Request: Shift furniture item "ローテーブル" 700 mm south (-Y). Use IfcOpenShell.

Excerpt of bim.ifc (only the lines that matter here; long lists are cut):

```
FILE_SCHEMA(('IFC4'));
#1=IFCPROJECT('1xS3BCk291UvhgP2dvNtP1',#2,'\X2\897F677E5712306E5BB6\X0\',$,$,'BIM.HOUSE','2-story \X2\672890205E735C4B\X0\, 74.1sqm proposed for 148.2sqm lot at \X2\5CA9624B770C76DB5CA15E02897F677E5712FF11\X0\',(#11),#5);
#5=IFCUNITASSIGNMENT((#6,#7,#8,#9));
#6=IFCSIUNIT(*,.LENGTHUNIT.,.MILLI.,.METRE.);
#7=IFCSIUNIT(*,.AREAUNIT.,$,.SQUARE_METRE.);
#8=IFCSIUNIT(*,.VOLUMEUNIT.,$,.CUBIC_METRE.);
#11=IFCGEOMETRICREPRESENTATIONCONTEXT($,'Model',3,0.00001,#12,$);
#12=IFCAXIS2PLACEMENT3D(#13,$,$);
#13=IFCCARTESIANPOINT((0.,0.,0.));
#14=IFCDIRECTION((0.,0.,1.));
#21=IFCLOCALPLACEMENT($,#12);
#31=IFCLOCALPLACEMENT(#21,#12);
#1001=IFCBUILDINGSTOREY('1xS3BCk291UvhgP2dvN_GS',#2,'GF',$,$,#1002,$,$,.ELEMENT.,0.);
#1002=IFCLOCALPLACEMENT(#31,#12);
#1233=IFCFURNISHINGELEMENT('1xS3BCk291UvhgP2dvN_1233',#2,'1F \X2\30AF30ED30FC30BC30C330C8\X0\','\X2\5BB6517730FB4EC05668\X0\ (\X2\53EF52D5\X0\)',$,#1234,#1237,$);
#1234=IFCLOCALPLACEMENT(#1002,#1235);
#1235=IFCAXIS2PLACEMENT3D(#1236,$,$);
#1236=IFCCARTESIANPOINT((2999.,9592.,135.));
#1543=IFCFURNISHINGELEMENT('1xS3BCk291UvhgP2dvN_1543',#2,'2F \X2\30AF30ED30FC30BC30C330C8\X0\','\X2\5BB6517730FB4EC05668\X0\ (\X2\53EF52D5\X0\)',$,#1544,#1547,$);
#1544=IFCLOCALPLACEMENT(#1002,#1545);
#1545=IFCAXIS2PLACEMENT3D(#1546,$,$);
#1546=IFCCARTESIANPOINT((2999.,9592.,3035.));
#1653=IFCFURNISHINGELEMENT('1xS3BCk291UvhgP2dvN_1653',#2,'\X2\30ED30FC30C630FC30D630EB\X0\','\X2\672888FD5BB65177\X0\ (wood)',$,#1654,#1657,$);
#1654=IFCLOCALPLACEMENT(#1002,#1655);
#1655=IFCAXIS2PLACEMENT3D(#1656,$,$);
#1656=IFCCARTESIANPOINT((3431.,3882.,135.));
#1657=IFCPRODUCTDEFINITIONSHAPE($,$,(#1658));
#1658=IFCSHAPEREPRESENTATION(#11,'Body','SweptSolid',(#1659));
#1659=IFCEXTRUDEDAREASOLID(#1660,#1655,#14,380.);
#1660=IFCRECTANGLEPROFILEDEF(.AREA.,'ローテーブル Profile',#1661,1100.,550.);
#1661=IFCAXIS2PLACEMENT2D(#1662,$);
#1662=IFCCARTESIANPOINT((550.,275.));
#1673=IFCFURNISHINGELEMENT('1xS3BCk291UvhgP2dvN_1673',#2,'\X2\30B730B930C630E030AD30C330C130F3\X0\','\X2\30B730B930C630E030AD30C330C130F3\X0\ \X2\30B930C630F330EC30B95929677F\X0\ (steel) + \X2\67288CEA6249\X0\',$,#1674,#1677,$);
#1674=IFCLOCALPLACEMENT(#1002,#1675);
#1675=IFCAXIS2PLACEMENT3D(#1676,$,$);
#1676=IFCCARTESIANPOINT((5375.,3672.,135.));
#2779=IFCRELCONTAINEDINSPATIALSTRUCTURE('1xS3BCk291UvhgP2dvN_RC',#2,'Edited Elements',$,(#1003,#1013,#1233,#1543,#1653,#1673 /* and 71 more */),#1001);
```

```python
import ifcopenshell
import ifcopenshell.api.geometry
import ifcopenshell.util.placement

model = ifcopenshell.open("bim.ifc")

item = model.by_guid("1xS3BCk291UvhgP2dvN_1653")
matrix = ifcopenshell.util.placement.get_local_placement(item.ObjectPlacement)
matrix[1, 3] -= 700.0
ifcopenshell.api.geometry.edit_object_placement(model, product=item, matrix=matrix, is_si=False)

print(ifcopenshell.util.placement.get_local_placement(item.ObjectPlacement).round(3) + 0.0)

model.write("bim_edited.ifc")
```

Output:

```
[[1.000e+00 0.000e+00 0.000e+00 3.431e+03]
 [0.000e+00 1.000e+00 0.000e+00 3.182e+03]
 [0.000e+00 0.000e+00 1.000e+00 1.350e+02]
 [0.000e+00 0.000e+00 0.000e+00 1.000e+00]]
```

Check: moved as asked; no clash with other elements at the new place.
